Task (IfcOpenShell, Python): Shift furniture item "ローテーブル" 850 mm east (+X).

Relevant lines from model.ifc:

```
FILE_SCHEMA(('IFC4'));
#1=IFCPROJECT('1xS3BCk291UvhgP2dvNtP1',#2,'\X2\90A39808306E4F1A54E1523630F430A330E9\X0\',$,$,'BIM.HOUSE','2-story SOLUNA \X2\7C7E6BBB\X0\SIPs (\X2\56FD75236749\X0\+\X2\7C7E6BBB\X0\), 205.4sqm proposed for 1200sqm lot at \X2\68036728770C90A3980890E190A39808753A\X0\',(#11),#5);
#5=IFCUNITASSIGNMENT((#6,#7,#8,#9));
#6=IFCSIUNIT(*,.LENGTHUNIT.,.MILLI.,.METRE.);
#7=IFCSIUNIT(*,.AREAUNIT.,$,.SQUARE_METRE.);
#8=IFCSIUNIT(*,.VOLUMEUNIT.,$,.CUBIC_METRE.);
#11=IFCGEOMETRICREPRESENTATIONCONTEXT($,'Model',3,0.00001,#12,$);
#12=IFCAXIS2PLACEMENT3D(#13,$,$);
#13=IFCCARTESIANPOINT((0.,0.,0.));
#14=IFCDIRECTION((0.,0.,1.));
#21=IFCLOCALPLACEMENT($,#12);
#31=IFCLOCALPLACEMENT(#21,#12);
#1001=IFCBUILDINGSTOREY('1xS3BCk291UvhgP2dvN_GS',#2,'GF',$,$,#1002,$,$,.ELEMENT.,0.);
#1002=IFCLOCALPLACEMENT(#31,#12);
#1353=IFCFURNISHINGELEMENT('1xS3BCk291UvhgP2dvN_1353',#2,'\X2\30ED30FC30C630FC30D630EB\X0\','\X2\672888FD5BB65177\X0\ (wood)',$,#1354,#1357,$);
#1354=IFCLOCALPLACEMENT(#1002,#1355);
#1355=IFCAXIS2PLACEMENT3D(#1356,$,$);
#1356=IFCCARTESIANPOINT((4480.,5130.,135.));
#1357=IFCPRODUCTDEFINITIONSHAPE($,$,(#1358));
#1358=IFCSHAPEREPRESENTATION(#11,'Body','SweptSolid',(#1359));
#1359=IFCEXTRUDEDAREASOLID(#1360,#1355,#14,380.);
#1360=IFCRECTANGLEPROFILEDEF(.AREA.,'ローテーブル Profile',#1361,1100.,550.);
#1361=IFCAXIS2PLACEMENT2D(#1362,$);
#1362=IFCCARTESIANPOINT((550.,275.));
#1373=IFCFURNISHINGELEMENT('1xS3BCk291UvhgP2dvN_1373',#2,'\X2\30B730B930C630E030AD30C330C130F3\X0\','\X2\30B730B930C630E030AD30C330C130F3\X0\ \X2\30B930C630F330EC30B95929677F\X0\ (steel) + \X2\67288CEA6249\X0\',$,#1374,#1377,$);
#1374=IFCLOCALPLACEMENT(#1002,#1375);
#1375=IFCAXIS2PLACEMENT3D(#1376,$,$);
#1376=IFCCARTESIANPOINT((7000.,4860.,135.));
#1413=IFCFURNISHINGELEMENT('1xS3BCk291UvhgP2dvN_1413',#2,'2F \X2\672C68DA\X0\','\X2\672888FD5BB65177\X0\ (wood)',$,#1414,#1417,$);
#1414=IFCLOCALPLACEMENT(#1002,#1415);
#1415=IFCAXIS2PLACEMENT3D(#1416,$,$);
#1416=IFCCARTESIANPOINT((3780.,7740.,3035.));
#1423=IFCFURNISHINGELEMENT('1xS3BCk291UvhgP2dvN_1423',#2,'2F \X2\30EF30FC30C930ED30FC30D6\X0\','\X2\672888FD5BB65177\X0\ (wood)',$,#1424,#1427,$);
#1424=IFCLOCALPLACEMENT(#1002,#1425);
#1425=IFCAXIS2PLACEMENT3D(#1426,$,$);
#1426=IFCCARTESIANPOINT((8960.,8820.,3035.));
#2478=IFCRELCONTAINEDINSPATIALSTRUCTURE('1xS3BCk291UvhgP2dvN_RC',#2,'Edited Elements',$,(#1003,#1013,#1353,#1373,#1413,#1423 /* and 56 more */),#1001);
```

```python
import ifcopenshell
import ifcopenshell.api.geometry
import ifcopenshell.util.placement
import ifcopenshell.util.unit

model = ifcopenshell.open("model.ifc")
unit_scale = ifcopenshell.util.unit.calculate_unit_scale(model)

item = model.by_guid("1xS3BCk291UvhgP2dvN_1353")
matrix = ifcopenshell.util.placement.get_local_placement(item.ObjectPlacement)
matrix[0, 3] += 0.85 / unit_scale
ifcopenshell.api.geometry.edit_object_placement(model, product=item, matrix=matrix, is_si=False)

print(ifcopenshell.util.placement.get_local_placement(item.ObjectPlacement).round(3) + 0.0)

model.write("model-out.ifc")
```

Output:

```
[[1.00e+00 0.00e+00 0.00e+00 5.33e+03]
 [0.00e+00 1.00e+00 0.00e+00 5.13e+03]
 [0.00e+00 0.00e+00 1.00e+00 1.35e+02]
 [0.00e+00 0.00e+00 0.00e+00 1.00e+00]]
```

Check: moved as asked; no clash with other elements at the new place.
